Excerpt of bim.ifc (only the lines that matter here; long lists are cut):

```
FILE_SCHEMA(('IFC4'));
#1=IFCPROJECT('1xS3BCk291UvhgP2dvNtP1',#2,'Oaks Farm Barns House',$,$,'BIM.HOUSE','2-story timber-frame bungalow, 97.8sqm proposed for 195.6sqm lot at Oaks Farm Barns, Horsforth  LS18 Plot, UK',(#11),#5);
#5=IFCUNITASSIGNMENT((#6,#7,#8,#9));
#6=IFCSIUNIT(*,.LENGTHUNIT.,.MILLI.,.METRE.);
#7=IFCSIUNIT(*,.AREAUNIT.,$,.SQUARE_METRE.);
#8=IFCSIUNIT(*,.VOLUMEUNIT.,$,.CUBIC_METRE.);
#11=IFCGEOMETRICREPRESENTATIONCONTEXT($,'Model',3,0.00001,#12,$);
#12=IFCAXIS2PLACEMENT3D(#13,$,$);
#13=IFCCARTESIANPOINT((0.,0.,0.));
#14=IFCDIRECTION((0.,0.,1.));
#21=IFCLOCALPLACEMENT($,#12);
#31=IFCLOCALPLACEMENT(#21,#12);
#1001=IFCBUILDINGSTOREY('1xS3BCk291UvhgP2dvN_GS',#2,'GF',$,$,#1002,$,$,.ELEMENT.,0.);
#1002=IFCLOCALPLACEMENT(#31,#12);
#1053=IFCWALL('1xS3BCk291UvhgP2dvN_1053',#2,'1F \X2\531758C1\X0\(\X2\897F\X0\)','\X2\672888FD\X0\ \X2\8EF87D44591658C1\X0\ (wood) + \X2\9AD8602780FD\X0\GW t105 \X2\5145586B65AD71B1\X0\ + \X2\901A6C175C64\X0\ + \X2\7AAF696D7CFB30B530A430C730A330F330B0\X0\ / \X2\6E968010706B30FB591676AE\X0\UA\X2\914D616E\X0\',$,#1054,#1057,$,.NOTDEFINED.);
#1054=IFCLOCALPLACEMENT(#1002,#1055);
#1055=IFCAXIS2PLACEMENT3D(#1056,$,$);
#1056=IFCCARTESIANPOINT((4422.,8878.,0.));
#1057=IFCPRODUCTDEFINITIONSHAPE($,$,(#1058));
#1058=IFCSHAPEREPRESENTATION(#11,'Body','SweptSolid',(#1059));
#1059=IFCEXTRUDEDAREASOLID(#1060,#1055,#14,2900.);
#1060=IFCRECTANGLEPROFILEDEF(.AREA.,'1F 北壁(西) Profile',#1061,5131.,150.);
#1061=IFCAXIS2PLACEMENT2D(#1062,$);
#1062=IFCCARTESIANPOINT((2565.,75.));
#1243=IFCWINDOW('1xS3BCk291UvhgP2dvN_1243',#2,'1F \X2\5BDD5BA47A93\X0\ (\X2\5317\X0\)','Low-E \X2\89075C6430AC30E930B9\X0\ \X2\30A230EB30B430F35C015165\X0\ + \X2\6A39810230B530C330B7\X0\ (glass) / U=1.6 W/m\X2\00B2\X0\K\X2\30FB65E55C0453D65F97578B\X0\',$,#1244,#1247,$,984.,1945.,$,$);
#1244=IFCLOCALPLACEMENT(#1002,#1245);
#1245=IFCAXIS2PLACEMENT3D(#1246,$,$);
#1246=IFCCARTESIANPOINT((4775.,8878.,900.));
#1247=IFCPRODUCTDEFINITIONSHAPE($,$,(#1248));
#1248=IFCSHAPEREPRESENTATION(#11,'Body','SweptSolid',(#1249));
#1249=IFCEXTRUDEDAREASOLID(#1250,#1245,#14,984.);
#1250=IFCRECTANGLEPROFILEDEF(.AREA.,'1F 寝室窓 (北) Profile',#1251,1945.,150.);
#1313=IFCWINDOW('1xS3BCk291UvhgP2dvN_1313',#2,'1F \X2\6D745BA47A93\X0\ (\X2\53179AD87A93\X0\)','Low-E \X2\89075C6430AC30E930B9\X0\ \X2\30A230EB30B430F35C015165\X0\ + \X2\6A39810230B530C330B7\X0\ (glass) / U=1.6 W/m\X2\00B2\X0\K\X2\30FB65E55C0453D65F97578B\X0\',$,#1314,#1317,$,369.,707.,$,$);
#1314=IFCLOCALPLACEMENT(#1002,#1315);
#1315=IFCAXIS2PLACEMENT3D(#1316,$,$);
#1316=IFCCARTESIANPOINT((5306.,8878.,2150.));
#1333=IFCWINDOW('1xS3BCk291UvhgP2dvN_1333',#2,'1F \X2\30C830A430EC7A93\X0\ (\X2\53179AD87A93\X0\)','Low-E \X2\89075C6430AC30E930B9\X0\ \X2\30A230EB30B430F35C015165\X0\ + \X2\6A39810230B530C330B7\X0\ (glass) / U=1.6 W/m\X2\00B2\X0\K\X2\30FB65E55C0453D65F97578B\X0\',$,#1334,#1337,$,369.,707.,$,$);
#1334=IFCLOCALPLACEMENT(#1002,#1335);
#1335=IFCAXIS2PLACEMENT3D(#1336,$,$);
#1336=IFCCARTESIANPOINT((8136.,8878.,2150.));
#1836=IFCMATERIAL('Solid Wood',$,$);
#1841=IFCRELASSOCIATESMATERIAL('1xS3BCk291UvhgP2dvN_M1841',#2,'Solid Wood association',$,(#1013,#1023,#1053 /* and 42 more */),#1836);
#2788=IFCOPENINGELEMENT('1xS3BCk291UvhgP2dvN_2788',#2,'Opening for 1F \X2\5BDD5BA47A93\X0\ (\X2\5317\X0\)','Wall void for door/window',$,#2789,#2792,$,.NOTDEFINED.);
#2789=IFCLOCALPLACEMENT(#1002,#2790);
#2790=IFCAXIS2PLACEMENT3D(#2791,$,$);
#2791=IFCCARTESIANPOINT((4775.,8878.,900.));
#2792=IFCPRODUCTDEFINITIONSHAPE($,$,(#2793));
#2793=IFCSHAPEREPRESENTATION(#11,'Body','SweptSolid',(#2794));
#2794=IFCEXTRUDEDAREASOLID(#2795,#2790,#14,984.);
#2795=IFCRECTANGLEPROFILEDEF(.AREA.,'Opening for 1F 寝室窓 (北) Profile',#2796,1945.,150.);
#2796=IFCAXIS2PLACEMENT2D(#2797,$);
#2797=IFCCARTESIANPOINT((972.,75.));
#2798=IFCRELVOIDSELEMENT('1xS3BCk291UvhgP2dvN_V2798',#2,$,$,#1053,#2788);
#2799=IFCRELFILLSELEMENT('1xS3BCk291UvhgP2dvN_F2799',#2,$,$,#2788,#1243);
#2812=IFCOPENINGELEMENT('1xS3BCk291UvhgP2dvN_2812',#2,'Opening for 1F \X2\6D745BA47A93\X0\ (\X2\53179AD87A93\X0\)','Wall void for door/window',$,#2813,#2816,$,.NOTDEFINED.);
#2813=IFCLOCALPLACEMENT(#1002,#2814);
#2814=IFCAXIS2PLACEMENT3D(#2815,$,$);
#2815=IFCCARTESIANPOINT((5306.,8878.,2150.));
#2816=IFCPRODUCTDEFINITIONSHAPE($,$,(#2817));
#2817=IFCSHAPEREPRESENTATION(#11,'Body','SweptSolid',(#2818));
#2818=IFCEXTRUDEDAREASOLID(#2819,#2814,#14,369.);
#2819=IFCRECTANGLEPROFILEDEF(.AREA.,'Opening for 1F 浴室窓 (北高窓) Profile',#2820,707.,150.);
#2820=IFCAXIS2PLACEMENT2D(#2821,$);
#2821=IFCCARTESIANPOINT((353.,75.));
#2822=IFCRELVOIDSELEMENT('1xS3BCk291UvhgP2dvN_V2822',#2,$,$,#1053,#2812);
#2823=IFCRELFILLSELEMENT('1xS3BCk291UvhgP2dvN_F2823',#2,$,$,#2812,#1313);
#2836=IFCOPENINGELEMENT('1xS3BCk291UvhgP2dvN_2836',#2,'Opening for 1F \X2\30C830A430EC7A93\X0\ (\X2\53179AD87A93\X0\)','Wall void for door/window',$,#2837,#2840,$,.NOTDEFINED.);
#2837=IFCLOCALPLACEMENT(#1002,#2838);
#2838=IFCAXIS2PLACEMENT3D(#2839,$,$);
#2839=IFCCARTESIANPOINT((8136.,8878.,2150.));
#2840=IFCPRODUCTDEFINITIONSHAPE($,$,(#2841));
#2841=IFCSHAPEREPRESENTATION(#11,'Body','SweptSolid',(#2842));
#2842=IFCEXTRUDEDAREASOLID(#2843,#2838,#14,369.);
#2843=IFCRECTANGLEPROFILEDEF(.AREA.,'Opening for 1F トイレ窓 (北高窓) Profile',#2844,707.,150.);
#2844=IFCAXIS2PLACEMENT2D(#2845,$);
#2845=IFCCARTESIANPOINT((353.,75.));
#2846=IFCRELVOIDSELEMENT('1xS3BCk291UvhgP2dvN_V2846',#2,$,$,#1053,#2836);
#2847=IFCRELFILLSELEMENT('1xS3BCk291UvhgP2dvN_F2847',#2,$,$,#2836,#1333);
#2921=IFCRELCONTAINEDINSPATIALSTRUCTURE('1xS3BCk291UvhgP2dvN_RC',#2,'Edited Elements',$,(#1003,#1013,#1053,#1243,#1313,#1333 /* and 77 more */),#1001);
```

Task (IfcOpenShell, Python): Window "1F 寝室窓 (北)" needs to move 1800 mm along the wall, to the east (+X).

```python
import ifcopenshell
import ifcopenshell.api.geometry
import ifcopenshell.util.placement
import ifcopenshell.util.unit

model = ifcopenshell.open("bim.ifc")
unit_scale = ifcopenshell.util.unit.calculate_unit_scale(model)

window = model.by_guid("1xS3BCk291UvhgP2dvN_1243")
opening = window.FillsVoids[0].RelatingOpeningElement
wall = opening.VoidsElements[0].RelatingBuildingElement

wall_matrix = ifcopenshell.util.placement.get_local_placement(wall.ObjectPlacement)
shift = wall_matrix[:3, 0] * 1.8 / unit_scale
before = ifcopenshell.util.placement.get_local_placement(window.ObjectPlacement)[:3, 3].copy()

# The window is not placed relative to its opening, so move both.
for product in (opening, window):
    matrix = ifcopenshell.util.placement.get_local_placement(product.ObjectPlacement)
    matrix[:3, 3] += shift
    ifcopenshell.api.geometry.edit_object_placement(model, product=product, matrix=matrix, is_si=False)

after = ifcopenshell.util.placement.get_local_placement(window.ObjectPlacement)[:3, 3]
print("window moved by", (after - before).round(3) + 0.0)

model.write("bim_rev.ifc")
```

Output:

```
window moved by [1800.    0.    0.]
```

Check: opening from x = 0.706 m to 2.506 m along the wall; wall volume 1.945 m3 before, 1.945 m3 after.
